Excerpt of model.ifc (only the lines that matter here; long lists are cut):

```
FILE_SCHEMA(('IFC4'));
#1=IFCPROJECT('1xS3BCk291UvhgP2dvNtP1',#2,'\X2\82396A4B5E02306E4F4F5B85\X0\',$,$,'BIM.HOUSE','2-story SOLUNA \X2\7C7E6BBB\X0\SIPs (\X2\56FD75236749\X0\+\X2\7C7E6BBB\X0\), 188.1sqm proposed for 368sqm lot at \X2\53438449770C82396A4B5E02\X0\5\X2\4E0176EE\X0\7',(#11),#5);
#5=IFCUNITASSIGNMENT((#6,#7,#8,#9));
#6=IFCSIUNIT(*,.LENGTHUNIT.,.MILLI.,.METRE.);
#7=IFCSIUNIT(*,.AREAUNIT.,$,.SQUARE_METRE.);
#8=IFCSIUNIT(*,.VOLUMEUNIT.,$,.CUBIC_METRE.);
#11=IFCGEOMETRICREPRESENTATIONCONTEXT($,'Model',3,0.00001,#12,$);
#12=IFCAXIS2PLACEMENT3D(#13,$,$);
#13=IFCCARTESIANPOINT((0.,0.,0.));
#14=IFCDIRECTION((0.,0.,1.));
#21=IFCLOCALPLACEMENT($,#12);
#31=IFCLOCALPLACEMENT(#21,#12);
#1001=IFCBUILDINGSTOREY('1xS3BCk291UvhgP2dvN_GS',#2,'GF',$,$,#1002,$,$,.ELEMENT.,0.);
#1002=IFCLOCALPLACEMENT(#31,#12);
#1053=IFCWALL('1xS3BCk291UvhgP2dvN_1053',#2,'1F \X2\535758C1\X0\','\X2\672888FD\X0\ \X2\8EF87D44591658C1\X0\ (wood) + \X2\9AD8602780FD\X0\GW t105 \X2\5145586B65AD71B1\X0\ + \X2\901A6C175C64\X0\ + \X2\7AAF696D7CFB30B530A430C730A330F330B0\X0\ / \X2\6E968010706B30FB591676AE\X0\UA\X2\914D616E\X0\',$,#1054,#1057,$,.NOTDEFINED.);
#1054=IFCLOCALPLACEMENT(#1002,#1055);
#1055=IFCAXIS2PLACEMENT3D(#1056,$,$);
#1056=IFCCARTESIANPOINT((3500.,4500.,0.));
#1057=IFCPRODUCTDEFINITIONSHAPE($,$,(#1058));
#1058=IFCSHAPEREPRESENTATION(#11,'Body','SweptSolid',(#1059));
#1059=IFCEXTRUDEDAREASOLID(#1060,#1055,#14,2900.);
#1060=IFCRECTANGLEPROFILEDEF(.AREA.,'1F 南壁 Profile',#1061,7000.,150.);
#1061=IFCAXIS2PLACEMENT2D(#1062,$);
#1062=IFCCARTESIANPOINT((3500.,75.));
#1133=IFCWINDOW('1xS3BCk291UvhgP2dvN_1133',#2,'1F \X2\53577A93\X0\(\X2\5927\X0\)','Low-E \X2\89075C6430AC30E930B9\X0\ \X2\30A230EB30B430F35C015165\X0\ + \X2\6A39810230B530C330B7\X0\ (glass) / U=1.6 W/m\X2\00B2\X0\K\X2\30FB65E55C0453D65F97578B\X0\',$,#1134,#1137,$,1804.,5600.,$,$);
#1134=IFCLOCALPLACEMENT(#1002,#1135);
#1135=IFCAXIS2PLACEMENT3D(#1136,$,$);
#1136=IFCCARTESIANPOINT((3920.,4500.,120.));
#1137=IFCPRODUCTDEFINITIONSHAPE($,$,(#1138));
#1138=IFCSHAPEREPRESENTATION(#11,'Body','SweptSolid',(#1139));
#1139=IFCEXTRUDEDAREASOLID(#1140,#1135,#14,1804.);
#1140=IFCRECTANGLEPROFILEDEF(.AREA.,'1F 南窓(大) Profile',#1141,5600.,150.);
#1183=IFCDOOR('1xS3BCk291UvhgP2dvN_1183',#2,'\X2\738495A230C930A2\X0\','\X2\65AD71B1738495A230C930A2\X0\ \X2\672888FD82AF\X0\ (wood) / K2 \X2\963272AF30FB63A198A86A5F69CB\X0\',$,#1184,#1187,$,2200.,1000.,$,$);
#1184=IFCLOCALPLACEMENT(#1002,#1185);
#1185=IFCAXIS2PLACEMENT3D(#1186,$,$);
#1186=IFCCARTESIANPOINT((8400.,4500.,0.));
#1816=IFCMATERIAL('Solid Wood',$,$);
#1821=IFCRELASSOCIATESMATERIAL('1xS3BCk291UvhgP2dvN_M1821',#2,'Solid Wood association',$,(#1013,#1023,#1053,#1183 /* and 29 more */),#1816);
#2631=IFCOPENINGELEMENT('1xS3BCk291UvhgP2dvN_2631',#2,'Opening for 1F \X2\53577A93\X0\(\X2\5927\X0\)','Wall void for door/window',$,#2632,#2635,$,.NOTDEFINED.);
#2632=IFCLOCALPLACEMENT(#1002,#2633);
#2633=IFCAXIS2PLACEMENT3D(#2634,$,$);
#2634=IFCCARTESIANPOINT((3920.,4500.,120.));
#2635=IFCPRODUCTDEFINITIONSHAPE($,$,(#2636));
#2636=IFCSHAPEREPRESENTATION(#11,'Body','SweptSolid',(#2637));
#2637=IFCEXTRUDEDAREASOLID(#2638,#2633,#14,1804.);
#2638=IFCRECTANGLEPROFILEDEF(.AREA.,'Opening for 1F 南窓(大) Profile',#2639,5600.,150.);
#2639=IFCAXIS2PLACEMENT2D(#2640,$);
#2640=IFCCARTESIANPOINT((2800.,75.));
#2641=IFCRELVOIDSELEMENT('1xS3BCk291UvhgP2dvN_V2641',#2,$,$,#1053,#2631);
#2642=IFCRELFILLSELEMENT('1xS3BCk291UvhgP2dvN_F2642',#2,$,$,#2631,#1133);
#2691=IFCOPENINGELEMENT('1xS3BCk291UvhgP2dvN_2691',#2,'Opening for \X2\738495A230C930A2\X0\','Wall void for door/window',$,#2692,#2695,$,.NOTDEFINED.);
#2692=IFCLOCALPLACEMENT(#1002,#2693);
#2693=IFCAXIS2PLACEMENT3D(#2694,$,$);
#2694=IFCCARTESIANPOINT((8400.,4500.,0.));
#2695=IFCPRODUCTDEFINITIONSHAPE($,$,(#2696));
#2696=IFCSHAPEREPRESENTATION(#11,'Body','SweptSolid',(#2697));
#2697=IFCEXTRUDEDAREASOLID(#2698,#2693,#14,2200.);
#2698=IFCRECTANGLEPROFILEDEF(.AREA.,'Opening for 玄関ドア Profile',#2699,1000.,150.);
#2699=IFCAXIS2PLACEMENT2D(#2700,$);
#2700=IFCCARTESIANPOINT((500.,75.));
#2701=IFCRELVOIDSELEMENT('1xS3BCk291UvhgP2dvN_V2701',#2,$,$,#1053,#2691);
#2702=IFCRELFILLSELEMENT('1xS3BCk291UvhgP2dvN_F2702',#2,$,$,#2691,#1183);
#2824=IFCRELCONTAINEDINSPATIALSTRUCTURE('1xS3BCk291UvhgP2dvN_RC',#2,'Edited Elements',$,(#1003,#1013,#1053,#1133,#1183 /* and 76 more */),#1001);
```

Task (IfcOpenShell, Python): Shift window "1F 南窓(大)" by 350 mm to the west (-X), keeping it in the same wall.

```python
import ifcopenshell
import ifcopenshell.api.geometry
import ifcopenshell.util.placement
import ifcopenshell.util.unit

model = ifcopenshell.open("model.ifc")
unit_scale = ifcopenshell.util.unit.calculate_unit_scale(model)

window = model.by_guid("1xS3BCk291UvhgP2dvN_1133")
opening = window.FillsVoids[0].RelatingOpeningElement
wall = opening.VoidsElements[0].RelatingBuildingElement

wall_matrix = ifcopenshell.util.placement.get_local_placement(wall.ObjectPlacement)
shift = wall_matrix[:3, 0] * -0.35 / unit_scale
before = ifcopenshell.util.placement.get_local_placement(window.ObjectPlacement)[:3, 3].copy()

# The window is not placed relative to its opening, so move both.
for product in (opening, window):
    matrix = ifcopenshell.util.placement.get_local_placement(product.ObjectPlacement)
    matrix[:3, 3] += shift
    ifcopenshell.api.geometry.edit_object_placement(model, product=product, matrix=matrix, is_si=False)

after = ifcopenshell.util.placement.get_local_placement(window.ObjectPlacement)[:3, 3]
print("window moved by", (after - before).round(3) + 0.0)

model.write("model_v2.ifc")
```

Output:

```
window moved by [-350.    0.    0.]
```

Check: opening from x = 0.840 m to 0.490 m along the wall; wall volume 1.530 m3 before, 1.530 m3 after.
